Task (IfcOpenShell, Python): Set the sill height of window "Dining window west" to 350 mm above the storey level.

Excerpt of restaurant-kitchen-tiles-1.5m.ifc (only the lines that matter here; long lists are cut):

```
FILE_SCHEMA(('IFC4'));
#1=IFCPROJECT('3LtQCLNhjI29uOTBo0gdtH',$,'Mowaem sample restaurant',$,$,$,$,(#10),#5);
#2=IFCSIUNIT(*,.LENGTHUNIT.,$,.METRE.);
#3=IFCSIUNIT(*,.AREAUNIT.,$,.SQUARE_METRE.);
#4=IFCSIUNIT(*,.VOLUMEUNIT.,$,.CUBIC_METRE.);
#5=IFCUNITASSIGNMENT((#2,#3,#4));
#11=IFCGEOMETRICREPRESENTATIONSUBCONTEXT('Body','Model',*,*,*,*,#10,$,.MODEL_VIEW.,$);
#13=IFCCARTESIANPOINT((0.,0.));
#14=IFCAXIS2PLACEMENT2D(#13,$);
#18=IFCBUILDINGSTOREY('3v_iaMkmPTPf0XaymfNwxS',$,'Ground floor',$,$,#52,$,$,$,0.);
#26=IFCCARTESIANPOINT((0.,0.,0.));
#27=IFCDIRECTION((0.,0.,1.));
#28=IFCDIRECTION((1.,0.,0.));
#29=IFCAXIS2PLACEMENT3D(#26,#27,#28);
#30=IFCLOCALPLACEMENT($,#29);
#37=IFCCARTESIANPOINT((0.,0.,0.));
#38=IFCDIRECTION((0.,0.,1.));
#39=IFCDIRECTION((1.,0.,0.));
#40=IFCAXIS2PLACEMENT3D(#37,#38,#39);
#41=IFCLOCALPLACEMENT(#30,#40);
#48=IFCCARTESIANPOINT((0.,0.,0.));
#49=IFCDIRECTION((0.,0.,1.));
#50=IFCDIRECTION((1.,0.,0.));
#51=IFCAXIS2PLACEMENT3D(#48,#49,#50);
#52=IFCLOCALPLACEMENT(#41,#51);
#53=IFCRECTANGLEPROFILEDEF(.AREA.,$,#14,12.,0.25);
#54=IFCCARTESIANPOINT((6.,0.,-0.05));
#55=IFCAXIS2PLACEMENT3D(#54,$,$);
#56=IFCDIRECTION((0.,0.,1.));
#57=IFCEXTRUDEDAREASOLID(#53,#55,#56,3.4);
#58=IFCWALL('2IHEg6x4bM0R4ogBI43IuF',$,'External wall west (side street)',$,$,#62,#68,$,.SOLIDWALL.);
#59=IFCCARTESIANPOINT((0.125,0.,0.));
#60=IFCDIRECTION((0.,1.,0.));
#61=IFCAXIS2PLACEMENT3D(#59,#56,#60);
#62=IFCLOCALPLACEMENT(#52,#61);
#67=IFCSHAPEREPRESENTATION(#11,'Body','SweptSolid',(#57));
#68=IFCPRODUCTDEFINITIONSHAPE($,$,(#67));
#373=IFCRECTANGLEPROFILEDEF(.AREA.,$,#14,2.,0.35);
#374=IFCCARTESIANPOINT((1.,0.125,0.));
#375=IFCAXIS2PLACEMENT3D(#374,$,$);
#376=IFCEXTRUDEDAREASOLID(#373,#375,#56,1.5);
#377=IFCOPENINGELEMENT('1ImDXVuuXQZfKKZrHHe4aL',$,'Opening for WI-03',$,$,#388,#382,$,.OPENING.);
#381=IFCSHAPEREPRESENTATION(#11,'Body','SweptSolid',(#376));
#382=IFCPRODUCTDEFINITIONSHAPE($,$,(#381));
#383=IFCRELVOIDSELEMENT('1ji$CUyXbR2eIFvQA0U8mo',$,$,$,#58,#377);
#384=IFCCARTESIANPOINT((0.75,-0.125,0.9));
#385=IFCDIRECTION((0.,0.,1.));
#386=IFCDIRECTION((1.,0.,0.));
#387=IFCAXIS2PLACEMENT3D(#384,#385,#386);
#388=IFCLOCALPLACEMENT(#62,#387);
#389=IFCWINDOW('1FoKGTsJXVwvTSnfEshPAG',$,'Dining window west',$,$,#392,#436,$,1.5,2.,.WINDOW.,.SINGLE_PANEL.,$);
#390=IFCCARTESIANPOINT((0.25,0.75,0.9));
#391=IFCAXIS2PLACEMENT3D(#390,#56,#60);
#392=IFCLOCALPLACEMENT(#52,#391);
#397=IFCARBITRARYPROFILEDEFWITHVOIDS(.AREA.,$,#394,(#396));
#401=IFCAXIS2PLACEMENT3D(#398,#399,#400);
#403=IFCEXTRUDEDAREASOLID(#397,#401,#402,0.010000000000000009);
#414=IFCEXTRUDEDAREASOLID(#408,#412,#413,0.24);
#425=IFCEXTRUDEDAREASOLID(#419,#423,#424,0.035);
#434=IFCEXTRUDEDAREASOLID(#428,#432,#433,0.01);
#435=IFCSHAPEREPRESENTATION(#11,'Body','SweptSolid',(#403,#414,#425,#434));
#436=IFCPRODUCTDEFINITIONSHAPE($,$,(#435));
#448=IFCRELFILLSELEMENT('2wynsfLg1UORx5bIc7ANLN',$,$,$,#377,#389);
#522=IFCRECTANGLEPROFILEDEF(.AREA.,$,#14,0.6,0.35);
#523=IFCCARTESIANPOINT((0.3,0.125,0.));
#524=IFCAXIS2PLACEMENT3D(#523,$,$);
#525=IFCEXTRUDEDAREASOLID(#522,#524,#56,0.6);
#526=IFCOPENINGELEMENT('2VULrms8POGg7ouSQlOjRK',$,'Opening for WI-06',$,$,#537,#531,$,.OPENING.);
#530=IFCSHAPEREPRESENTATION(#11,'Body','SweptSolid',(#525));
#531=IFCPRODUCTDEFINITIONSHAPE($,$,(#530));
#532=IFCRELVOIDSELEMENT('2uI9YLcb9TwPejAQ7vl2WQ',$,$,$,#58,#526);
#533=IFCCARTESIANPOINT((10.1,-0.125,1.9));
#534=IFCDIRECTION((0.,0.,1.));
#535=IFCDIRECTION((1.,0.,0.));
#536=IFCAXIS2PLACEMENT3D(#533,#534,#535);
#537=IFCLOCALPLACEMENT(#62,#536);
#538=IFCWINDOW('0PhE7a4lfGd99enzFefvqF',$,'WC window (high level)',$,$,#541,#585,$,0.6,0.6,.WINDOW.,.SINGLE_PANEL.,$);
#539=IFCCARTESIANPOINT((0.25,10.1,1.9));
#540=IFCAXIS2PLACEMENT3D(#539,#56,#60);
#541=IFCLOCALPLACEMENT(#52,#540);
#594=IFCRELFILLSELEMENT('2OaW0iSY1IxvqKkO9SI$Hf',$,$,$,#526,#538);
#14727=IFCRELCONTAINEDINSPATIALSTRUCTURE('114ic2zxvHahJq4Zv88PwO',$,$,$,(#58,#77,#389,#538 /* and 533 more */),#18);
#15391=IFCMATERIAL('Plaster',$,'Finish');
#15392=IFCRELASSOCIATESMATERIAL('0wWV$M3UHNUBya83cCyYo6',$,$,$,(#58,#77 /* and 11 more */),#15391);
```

```python
import numpy as np
import ifcopenshell
import ifcopenshell.api.geometry
import ifcopenshell.geom
import ifcopenshell.util.element
import ifcopenshell.util.placement
import ifcopenshell.util.shape
import ifcopenshell.util.unit

model = ifcopenshell.open("restaurant-kitchen-tiles-1.5m.ifc")
unit_scale = ifcopenshell.util.unit.calculate_unit_scale(model)

window = model.by_guid("1FoKGTsJXVwvTSnfEshPAG")
opening = window.FillsVoids[0].RelatingOpeningElement
storey = ifcopenshell.util.element.get_container(window, ifc_class="IfcBuildingStorey")
level = ifcopenshell.util.placement.get_local_placement(storey.ObjectPlacement)[2, 3]

# The opening's origin need not be at the sill, so measure its lowest point.
shape = ifcopenshell.geom.create_shape(ifcopenshell.geom.settings(), opening)
bottom = ifcopenshell.util.shape.get_shape_bottom_elevation(shape, shape.geometry) / unit_scale
dz = level + 0.35 / unit_scale - bottom

shift = np.array([0.0, 0.0, dz])
# The window is not placed relative to its opening, so move both.
for product in (opening, window):
    matrix = ifcopenshell.util.placement.get_local_placement(product.ObjectPlacement)
    matrix[:3, 3] += shift
    ifcopenshell.api.geometry.edit_object_placement(model, product=product, matrix=matrix, is_si=False)

print(f"moved by {dz * unit_scale:+.3f} m")

model.write("restaurant-kitchen-tiles-1.5m_v2.ifc")
```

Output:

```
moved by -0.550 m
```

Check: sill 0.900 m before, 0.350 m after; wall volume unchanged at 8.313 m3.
